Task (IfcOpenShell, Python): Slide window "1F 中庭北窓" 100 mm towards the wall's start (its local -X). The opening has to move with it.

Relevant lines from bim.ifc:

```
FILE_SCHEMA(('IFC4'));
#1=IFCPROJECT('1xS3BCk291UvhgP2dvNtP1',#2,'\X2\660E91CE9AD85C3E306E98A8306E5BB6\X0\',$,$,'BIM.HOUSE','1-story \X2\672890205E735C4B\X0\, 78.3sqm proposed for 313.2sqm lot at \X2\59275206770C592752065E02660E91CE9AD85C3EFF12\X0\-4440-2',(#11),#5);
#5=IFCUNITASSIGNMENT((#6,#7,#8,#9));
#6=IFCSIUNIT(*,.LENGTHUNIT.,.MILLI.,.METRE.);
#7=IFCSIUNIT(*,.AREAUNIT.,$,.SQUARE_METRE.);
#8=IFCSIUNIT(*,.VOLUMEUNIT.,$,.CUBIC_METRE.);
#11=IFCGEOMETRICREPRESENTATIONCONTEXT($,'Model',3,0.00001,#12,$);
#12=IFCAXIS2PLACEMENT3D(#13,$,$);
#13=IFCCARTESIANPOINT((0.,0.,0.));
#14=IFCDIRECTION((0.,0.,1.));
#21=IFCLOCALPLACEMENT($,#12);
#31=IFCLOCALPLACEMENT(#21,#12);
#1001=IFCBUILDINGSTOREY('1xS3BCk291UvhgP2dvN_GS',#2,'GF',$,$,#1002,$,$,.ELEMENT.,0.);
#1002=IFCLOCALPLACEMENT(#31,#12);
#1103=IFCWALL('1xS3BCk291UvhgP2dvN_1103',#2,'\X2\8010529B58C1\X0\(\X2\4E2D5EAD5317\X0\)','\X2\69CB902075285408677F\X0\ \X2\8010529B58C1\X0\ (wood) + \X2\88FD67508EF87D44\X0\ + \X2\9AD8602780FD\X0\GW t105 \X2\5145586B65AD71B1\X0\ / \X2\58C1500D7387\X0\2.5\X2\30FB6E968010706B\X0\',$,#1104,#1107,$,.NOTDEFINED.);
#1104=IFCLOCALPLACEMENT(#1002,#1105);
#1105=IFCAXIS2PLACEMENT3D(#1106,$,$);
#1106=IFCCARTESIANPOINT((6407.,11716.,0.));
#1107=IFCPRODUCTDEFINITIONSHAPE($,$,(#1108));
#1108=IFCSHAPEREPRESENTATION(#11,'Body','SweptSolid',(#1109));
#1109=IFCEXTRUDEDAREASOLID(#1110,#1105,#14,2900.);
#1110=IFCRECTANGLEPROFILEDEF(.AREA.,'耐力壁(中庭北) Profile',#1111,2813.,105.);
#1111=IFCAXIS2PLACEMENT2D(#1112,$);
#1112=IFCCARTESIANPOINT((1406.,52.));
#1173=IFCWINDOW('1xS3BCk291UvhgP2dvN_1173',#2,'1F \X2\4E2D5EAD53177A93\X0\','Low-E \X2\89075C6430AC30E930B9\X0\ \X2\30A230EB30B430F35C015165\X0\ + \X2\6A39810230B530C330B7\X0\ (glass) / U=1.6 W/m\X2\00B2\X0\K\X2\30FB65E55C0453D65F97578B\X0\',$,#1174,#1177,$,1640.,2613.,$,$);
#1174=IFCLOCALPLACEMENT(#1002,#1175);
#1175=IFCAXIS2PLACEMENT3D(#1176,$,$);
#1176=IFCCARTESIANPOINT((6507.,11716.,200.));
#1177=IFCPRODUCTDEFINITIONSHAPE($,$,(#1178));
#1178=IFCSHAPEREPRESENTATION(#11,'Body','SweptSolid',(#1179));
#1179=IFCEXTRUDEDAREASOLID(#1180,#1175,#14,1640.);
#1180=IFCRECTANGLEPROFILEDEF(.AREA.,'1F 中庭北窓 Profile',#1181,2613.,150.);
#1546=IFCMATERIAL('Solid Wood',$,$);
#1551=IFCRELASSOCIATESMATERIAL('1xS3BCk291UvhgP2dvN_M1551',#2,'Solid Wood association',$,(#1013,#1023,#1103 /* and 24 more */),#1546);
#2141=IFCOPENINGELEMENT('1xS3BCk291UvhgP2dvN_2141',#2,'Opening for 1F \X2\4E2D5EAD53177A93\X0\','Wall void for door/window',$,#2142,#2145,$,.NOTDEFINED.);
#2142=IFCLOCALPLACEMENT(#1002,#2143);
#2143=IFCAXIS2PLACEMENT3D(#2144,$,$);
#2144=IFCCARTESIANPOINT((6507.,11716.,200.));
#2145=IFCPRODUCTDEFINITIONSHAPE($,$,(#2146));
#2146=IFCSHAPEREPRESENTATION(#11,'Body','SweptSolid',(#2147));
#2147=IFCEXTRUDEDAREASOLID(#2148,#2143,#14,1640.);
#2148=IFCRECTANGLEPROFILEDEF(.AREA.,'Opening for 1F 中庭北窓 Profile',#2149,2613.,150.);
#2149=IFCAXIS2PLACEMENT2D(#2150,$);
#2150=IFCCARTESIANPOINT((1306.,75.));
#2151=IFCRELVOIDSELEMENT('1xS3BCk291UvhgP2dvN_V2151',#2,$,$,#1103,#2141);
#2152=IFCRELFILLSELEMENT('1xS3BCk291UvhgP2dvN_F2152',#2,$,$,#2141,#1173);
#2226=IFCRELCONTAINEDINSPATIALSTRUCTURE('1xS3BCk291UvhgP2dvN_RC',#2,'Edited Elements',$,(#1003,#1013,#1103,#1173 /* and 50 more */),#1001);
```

```python
import ifcopenshell
import ifcopenshell.api.geometry
import ifcopenshell.util.placement
import ifcopenshell.util.unit

model = ifcopenshell.open("bim.ifc")
unit_scale = ifcopenshell.util.unit.calculate_unit_scale(model)

window = model.by_id(1173)
opening = window.FillsVoids[0].RelatingOpeningElement
wall = opening.VoidsElements[0].RelatingBuildingElement

wall_matrix = ifcopenshell.util.placement.get_local_placement(wall.ObjectPlacement)
shift = wall_matrix[:3, 0] * -0.1 / unit_scale
before = ifcopenshell.util.placement.get_local_placement(window.ObjectPlacement)[:3, 3].copy()

# The window is not placed relative to its opening, so move both.
for product in (opening, window):
    matrix = ifcopenshell.util.placement.get_local_placement(product.ObjectPlacement)
    matrix[:3, 3] += shift
    ifcopenshell.api.geometry.edit_object_placement(model, product=product, matrix=matrix, is_si=False)

after = ifcopenshell.util.placement.get_local_placement(window.ObjectPlacement)[:3, 3]
print("window moved by", (after - before).round(3) + 0.0)

model.write("bim_edited.ifc")
```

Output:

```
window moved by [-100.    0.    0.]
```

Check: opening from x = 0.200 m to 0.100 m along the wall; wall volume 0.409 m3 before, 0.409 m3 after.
